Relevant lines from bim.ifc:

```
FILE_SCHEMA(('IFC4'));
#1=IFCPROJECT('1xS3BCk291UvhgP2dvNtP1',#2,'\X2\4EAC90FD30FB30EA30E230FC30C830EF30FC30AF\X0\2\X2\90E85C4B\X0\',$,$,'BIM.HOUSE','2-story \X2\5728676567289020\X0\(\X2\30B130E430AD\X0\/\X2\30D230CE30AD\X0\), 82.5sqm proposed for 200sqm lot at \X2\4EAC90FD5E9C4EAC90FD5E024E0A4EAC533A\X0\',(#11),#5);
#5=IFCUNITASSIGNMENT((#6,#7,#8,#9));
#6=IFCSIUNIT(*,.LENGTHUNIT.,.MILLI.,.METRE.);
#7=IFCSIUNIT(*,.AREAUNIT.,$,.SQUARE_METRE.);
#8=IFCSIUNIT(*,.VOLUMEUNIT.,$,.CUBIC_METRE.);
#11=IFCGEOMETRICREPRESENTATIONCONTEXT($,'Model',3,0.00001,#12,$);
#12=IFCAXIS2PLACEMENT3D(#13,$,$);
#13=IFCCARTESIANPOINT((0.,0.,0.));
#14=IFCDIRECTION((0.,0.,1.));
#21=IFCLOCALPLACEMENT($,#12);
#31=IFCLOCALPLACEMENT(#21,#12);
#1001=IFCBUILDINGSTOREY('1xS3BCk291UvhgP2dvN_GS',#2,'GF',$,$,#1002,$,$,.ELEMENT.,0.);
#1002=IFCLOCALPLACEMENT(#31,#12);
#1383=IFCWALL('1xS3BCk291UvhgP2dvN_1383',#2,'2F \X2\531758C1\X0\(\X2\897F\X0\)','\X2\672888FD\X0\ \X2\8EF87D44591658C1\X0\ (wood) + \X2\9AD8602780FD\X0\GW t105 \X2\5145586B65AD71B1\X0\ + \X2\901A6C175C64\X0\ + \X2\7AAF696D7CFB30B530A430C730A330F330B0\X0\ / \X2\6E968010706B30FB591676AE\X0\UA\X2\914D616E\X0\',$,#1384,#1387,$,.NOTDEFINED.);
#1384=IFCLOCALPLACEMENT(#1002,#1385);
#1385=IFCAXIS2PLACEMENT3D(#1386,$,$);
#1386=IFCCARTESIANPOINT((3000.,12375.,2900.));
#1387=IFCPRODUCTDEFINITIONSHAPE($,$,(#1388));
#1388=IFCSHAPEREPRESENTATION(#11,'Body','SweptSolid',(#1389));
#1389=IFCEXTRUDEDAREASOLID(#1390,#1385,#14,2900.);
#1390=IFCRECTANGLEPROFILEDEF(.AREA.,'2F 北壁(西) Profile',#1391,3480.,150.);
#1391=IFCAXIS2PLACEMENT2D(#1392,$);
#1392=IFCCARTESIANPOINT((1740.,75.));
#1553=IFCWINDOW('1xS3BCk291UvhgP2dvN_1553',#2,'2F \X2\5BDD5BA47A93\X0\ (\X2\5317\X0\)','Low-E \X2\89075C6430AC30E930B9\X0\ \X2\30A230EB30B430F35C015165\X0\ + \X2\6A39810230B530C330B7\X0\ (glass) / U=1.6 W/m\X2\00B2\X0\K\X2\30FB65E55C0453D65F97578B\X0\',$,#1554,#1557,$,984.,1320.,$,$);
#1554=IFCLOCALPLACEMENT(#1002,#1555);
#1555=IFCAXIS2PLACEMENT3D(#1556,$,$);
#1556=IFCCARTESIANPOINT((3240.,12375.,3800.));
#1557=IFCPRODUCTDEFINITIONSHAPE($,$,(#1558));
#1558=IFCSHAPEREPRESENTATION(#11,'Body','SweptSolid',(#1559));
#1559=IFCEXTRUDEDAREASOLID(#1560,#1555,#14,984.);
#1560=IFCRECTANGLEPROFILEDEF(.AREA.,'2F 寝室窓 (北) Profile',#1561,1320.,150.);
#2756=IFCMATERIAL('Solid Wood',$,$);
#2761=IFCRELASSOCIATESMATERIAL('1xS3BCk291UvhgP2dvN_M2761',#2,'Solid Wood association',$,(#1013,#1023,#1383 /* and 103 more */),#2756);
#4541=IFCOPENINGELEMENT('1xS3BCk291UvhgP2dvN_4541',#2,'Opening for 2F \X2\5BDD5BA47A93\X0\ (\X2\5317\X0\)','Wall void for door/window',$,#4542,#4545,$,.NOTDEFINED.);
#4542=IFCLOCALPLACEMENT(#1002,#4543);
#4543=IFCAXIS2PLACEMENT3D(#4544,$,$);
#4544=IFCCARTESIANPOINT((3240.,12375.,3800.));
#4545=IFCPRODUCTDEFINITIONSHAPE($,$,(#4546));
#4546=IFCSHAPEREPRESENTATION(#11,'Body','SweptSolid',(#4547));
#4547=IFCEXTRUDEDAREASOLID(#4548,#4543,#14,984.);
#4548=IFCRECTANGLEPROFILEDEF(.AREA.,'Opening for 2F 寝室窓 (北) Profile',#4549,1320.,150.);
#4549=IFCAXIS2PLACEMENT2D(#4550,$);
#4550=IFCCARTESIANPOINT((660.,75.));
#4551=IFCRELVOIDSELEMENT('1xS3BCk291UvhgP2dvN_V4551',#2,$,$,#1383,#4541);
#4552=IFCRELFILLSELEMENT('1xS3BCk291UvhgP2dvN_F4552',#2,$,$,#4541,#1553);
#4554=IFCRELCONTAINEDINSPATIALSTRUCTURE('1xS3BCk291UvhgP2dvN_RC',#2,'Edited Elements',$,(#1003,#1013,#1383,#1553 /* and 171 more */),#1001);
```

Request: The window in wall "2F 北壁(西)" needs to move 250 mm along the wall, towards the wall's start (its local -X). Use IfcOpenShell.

```python
import ifcopenshell
import ifcopenshell.api.geometry
import ifcopenshell.util.placement
import ifcopenshell.util.unit

model = ifcopenshell.open("bim.ifc")
unit_scale = ifcopenshell.util.unit.calculate_unit_scale(model)

window = model.by_guid("1xS3BCk291UvhgP2dvN_1553")
opening = window.FillsVoids[0].RelatingOpeningElement
wall = opening.VoidsElements[0].RelatingBuildingElement

wall_matrix = ifcopenshell.util.placement.get_local_placement(wall.ObjectPlacement)
shift = wall_matrix[:3, 0] * -0.25 / unit_scale
before = ifcopenshell.util.placement.get_local_placement(window.ObjectPlacement)[:3, 3].copy()

# The window is not placed relative to its opening, so move both.
for product in (opening, window):
    matrix = ifcopenshell.util.placement.get_local_placement(product.ObjectPlacement)
    matrix[:3, 3] += shift
    ifcopenshell.api.geometry.edit_object_placement(model, product=product, matrix=matrix, is_si=False)

after = ifcopenshell.util.placement.get_local_placement(window.ObjectPlacement)[:3, 3]
print("window moved by", (after - before).round(3) + 0.0)

model.write("bim_rev.ifc")
```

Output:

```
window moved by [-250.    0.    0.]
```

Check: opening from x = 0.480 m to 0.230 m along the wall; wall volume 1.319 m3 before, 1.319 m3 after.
